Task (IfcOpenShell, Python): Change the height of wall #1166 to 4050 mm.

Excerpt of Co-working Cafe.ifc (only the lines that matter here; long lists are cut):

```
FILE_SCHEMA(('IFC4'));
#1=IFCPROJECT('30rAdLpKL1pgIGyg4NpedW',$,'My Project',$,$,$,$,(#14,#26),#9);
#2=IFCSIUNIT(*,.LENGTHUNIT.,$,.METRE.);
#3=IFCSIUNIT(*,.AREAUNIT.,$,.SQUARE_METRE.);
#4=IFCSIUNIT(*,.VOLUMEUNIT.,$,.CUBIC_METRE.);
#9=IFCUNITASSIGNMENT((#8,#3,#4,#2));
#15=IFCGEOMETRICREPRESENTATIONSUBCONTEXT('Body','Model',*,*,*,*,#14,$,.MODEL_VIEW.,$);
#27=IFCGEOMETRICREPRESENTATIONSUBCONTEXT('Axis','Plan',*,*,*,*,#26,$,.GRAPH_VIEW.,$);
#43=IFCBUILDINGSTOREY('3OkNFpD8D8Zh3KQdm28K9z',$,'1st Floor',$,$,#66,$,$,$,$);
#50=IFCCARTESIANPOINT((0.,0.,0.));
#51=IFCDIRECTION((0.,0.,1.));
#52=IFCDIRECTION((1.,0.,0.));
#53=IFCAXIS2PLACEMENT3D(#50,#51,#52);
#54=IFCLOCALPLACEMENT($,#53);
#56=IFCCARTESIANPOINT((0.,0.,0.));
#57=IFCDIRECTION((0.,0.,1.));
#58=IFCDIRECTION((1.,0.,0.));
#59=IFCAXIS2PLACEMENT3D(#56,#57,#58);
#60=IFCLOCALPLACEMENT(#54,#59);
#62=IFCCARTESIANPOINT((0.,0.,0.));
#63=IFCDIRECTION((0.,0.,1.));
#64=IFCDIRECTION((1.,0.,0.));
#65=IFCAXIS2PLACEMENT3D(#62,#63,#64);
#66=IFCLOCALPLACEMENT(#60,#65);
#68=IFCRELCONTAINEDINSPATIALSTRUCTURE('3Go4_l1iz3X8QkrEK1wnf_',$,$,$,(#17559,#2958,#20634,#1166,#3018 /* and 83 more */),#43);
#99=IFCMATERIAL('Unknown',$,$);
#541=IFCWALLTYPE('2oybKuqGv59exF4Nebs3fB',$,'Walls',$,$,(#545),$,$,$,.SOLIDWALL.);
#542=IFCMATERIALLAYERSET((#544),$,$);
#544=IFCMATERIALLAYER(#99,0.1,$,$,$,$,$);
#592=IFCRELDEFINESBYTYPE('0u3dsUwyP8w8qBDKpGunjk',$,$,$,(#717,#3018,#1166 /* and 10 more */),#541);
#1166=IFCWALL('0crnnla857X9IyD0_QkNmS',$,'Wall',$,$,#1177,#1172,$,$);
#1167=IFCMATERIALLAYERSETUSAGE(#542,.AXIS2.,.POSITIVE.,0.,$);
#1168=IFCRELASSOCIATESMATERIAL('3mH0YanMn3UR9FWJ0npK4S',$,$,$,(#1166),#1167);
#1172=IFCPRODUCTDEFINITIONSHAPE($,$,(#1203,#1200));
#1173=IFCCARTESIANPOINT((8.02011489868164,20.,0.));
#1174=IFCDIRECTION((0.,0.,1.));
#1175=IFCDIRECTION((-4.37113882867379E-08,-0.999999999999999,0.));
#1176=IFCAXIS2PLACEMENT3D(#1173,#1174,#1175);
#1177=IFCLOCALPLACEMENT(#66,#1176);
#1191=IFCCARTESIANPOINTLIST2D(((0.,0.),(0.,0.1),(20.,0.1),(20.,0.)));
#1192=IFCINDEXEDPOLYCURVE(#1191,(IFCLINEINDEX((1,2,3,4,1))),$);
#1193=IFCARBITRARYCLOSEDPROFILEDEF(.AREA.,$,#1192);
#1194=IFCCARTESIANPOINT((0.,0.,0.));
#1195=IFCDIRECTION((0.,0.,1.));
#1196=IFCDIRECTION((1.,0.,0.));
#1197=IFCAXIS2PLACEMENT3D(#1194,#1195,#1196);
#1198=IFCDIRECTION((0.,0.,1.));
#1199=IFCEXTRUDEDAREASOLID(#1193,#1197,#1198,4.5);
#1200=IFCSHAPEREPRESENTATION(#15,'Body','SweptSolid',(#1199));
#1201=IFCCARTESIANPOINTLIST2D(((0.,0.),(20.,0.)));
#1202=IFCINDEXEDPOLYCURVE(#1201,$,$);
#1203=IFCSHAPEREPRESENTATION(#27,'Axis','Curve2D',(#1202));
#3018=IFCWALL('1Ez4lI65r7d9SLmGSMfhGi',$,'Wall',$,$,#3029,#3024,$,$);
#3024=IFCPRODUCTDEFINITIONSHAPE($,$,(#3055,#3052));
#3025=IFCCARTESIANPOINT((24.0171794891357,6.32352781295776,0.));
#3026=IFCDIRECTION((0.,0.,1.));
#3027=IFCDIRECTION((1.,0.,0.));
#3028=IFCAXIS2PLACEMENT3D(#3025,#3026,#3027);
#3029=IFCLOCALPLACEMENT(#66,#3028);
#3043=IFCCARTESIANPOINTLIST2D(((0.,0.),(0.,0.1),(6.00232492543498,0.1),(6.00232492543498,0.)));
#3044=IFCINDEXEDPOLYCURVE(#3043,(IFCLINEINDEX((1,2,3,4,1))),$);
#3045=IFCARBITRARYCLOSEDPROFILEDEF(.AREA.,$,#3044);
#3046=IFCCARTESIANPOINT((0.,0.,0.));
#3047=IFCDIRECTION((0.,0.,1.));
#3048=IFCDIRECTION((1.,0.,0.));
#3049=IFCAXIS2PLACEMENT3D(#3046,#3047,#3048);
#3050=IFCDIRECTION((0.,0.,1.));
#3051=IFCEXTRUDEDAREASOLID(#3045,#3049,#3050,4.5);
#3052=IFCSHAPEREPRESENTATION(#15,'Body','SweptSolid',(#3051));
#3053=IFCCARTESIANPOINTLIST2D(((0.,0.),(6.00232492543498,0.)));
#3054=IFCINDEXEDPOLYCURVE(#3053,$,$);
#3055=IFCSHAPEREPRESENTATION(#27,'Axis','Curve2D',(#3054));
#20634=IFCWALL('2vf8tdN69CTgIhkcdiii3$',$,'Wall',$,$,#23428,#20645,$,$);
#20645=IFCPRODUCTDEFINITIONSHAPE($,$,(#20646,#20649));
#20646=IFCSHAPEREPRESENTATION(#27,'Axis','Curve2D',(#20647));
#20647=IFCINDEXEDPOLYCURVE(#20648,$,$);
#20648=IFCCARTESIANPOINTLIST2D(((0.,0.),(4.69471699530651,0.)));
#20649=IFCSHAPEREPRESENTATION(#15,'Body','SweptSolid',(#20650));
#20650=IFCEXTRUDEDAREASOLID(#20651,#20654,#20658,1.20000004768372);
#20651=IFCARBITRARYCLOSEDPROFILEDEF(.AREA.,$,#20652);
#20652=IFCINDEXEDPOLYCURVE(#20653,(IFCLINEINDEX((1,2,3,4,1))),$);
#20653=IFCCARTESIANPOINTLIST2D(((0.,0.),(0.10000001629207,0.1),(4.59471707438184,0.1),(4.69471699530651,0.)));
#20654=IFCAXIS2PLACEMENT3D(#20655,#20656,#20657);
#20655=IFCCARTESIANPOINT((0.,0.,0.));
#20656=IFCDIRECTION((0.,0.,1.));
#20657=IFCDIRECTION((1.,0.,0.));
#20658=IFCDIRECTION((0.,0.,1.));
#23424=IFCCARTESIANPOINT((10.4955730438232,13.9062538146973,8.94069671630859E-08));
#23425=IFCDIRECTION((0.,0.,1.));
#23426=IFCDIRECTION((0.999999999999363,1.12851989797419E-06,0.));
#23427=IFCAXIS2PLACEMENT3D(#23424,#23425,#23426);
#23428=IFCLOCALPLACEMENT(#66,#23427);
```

```python
import ifcopenshell
import ifcopenshell.geom
import ifcopenshell.util.representation
import ifcopenshell.util.shape
import ifcopenshell.util.unit

model = ifcopenshell.open("Co-working Cafe.ifc")
unit_scale = ifcopenshell.util.unit.calculate_unit_scale(model)
settings = ifcopenshell.geom.settings()


def volume(element):
    """Net volume in cubic metres, openings subtracted."""
    shape = ifcopenshell.geom.create_shape(settings, element)
    return ifcopenshell.util.shape.get_volume(shape.geometry)


wall = model.by_guid("0crnnla857X9IyD0_QkNmS")
before = volume(wall)

body = ifcopenshell.util.representation.get_representation(wall, "Model", "Body")
solid = body.Items[0]
old_height = solid.Depth
solid.Depth = 4.05 / unit_scale
after = volume(wall)

print(f"height {old_height:g} -> {solid.Depth:g}, volume {before:.3f} -> {after:.3f} m3")

model.write("Co-working Cafe_v2.ifc")
```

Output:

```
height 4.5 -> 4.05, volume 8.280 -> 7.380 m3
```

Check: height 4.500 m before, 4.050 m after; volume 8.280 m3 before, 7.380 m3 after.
